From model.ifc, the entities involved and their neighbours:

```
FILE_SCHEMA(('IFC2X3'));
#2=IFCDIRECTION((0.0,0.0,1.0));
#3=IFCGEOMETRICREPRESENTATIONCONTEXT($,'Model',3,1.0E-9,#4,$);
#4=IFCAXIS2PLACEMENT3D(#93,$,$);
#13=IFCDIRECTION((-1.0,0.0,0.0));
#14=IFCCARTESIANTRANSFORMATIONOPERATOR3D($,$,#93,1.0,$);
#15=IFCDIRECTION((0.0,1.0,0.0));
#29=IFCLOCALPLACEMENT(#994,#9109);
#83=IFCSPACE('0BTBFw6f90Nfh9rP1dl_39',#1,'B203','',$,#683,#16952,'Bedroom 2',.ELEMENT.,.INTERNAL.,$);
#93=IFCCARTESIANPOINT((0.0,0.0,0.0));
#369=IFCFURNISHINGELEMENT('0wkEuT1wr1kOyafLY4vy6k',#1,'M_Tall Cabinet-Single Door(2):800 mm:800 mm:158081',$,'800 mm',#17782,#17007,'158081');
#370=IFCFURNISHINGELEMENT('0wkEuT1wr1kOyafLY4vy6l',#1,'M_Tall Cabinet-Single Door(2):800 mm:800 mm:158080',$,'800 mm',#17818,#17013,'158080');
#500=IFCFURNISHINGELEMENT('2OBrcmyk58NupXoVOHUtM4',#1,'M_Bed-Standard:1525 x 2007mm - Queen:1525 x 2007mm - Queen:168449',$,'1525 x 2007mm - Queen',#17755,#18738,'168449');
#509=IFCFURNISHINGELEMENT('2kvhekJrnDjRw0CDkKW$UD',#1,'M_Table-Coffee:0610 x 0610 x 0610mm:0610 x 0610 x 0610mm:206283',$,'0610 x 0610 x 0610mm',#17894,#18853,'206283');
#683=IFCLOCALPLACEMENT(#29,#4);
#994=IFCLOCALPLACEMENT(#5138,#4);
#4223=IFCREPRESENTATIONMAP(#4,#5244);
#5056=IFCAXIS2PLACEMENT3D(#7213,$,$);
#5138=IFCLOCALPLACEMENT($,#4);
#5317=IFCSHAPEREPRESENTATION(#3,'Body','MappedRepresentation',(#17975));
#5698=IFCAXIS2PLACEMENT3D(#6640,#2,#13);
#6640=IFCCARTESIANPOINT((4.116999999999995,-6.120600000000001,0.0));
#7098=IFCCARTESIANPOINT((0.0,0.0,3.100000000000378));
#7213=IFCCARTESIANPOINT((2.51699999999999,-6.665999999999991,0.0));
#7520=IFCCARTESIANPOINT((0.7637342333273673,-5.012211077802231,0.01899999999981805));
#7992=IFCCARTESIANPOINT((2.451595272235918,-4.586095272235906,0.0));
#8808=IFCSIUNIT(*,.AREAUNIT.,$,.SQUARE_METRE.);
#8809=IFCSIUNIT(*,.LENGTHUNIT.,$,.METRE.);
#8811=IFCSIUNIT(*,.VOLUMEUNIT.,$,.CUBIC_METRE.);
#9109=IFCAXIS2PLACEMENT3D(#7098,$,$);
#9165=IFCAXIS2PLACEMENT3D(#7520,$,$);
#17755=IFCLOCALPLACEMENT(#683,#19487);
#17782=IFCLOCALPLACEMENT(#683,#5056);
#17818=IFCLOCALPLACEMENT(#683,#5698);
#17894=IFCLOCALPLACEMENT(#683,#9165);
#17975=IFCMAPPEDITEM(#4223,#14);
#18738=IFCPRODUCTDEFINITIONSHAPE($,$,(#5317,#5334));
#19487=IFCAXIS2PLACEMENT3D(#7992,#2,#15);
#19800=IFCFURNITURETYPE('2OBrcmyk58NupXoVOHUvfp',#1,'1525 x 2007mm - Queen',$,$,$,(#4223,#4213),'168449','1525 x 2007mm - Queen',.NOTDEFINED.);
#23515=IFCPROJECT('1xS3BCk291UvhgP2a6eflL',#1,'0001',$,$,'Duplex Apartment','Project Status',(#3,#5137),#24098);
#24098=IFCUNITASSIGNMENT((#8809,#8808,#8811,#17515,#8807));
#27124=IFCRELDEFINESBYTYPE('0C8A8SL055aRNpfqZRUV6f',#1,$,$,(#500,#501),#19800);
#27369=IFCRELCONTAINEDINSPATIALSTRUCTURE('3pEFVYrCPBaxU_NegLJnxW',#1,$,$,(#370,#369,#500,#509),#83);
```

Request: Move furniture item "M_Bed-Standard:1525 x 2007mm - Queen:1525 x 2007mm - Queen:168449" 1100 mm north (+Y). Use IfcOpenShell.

```python
import ifcopenshell
import ifcopenshell.api.geometry
import ifcopenshell.util.placement
import ifcopenshell.util.unit

model = ifcopenshell.open("model.ifc")
unit_scale = ifcopenshell.util.unit.calculate_unit_scale(model)

item = model.by_guid("2OBrcmyk58NupXoVOHUtM4")
matrix = ifcopenshell.util.placement.get_local_placement(item.ObjectPlacement)
matrix[1, 3] += 1.1 / unit_scale
ifcopenshell.api.geometry.edit_object_placement(model, product=item, matrix=matrix, is_si=False)

print(ifcopenshell.util.placement.get_local_placement(item.ObjectPlacement).round(3) + 0.0)

model.write("model-out.ifc")
```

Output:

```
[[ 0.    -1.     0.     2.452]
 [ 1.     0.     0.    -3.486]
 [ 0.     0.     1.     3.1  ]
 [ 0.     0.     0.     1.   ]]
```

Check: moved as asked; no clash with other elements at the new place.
